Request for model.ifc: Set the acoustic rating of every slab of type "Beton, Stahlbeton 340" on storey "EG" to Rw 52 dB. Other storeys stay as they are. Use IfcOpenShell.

First a look at what the model holds.

```python
import ifcopenshell
import ifcopenshell.util.element

model = ifcopenshell.open("model.ifc")
print(model.schema)
storey = next(s for s in model.by_type("IfcBuildingStorey") if s.Name == "EG")
slabs = [e for e in ifcopenshell.util.element.get_decomposition(storey) if e.is_a("IfcSlab")]
seen = {}
for e in slabs:
    element_type = ifcopenshell.util.element.get_type(e)
    key = (element_type.Name if element_type != e and element_type else None, ifcopenshell.util.element.get_pset(e, "Pset_SlabCommon", "AcousticRating"))
    seen[key] = seen.get(key, 0) + 1
for (name, value), count in sorted(seen.items(), key=str):
    print(count, "x", name, "|", value)
```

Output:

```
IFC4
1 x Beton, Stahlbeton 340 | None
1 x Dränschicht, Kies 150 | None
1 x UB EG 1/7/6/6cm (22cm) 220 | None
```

```python
import ifcopenshell
import ifcopenshell.api.pset
import ifcopenshell.util.element

model = ifcopenshell.open("model.ifc")

storey = next(s for s in model.by_type("IfcBuildingStorey") if s.Name == "EG")
slabs = [e for e in ifcopenshell.util.element.get_decomposition(storey) if e.is_a("IfcSlab")]

count = 0
for e in slabs:
    element_type = ifcopenshell.util.element.get_type(e)
    if element_type in (None, e) or element_type.Name != "Beton, Stahlbeton 340":
        continue
    # add_pset returns the element's existing set when there is one.
    pset = ifcopenshell.api.pset.add_pset(model, product=e, name="Pset_SlabCommon")
    ifcopenshell.api.pset.edit_pset(model, pset=pset, properties={"AcousticRating": "Rw 52 dB"})
    count += 1

print(count, "slabs updated")

model.write("model_rev.ifc")
```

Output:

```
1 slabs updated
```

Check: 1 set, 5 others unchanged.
